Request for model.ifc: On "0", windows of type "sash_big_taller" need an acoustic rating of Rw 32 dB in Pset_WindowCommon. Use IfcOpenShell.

First a look at what the model holds.

```python
import ifcopenshell
import ifcopenshell.util.element

model = ifcopenshell.open("model.ifc")
print(model.schema)
storey = next(s for s in model.by_type("IfcBuildingStorey") if s.Name == "0")
windows = [e for e in ifcopenshell.util.element.get_decomposition(storey) if e.is_a("IfcWindow")]
seen = {}
for e in windows:
    element_type = ifcopenshell.util.element.get_type(e)
    key = (element_type.Name if element_type != e and element_type else None, ifcopenshell.util.element.get_pset(e, "Pset_WindowCommon", "AcousticRating"))
    seen[key] = seen.get(key, 0) + 1
for (name, value), count in sorted(seen.items(), key=str):
    print(count, "x", name, "|", value)
```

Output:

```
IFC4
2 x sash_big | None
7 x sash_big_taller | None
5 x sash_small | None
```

```python
import ifcopenshell
import ifcopenshell.api.pset
import ifcopenshell.util.element

model = ifcopenshell.open("model.ifc")

storey = next(s for s in model.by_type("IfcBuildingStorey") if s.Name == "0")
windows = [e for e in ifcopenshell.util.element.get_decomposition(storey) if e.is_a("IfcWindow")]

count = 0
for e in windows:
    element_type = ifcopenshell.util.element.get_type(e)
    if element_type in (None, e) or element_type.Name != "sash_big_taller":
        continue
    # add_pset returns the element's existing set when there is one.
    pset = ifcopenshell.api.pset.add_pset(model, product=e, name="Pset_WindowCommon")
    ifcopenshell.api.pset.edit_pset(model, pset=pset, properties={"AcousticRating": "Rw 32 dB"})
    count += 1

print(count, "windows updated")

model.write("model_edited.ifc")
```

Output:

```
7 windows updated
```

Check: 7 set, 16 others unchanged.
